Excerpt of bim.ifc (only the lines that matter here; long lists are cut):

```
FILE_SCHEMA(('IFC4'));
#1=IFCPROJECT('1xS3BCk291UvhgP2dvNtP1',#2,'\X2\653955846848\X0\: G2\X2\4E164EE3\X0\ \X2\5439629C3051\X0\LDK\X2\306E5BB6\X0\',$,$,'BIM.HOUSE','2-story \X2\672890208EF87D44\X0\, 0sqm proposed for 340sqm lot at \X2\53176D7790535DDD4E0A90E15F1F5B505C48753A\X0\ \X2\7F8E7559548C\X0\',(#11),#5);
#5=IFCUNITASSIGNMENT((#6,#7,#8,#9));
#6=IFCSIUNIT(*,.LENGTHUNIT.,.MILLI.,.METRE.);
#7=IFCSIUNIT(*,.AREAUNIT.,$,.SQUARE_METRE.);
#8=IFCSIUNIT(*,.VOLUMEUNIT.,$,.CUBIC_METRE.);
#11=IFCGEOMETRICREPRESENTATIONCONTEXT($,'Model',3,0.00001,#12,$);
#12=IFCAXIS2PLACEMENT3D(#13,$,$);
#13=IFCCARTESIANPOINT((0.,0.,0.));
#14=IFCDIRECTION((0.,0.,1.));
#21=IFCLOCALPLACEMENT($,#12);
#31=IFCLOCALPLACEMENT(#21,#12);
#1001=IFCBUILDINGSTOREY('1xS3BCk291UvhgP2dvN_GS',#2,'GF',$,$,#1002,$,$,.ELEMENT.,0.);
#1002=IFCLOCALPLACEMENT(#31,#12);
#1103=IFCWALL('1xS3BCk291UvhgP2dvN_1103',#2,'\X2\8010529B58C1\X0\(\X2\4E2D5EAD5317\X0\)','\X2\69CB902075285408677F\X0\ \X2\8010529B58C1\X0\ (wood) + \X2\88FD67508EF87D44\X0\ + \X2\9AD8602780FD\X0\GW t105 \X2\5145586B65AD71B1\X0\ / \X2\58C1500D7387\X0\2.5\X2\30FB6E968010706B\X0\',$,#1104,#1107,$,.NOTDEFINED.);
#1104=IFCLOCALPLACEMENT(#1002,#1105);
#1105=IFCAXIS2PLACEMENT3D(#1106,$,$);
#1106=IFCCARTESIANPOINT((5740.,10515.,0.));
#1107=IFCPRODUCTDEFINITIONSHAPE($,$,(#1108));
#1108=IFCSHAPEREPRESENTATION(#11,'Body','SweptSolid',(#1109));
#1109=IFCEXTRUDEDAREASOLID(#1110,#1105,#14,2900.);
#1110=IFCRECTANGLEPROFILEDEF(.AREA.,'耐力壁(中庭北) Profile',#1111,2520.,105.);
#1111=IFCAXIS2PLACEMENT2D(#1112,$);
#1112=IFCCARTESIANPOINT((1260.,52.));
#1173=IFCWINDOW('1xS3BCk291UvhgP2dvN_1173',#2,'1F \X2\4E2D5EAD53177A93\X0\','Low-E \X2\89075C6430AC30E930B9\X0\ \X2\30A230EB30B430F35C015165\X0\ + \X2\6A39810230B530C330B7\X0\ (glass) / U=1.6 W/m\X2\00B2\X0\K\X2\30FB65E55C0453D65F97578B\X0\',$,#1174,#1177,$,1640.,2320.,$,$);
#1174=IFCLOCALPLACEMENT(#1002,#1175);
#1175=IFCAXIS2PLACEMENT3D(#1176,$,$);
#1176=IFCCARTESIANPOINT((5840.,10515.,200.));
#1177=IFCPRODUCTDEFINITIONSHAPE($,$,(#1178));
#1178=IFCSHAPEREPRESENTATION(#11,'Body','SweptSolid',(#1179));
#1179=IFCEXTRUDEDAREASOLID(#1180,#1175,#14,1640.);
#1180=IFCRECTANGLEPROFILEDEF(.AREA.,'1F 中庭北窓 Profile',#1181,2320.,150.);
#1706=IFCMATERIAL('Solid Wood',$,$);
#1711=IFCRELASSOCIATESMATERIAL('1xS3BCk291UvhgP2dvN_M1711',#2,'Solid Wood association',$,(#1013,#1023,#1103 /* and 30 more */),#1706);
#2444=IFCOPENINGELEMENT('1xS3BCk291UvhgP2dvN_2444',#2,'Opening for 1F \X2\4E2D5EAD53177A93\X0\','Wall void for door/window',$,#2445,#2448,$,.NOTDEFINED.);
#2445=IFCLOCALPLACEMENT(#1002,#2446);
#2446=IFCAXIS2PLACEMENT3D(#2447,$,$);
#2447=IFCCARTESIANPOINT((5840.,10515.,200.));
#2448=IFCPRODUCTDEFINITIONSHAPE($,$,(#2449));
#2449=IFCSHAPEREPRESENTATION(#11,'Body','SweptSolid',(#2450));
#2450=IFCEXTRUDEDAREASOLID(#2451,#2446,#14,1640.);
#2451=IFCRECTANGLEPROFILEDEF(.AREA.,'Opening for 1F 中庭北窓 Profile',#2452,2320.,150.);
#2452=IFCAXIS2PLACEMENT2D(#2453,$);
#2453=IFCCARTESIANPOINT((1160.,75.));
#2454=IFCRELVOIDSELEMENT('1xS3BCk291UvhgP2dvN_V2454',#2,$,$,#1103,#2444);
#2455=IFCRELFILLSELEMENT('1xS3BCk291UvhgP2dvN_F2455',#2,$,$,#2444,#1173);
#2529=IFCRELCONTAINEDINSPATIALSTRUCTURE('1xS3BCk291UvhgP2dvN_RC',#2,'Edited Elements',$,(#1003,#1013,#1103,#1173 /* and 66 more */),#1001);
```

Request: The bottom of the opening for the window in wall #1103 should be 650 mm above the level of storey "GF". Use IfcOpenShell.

```python
import numpy as np
import ifcopenshell
import ifcopenshell.api.geometry
import ifcopenshell.geom
import ifcopenshell.util.element
import ifcopenshell.util.placement
import ifcopenshell.util.shape
import ifcopenshell.util.unit

model = ifcopenshell.open("bim.ifc")
unit_scale = ifcopenshell.util.unit.calculate_unit_scale(model)

window = model.by_guid("1xS3BCk291UvhgP2dvN_1173")
opening = window.FillsVoids[0].RelatingOpeningElement
storey = ifcopenshell.util.element.get_container(window, ifc_class="IfcBuildingStorey")
level = ifcopenshell.util.placement.get_local_placement(storey.ObjectPlacement)[2, 3]

# The opening's origin need not be at the sill, so measure its lowest point.
shape = ifcopenshell.geom.create_shape(ifcopenshell.geom.settings(), opening)
bottom = ifcopenshell.util.shape.get_shape_bottom_elevation(shape, shape.geometry) / unit_scale
dz = level + 0.65 / unit_scale - bottom

shift = np.array([0.0, 0.0, dz])
# The window is not placed relative to its opening, so move both.
for product in (opening, window):
    matrix = ifcopenshell.util.placement.get_local_placement(product.ObjectPlacement)
    matrix[:3, 3] += shift
    ifcopenshell.api.geometry.edit_object_placement(model, product=product, matrix=matrix, is_si=False)

print(f"moved by {dz * unit_scale:+.3f} m")

model.write("bim_edited.ifc")
```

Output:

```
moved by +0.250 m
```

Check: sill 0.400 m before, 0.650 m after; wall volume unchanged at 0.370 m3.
